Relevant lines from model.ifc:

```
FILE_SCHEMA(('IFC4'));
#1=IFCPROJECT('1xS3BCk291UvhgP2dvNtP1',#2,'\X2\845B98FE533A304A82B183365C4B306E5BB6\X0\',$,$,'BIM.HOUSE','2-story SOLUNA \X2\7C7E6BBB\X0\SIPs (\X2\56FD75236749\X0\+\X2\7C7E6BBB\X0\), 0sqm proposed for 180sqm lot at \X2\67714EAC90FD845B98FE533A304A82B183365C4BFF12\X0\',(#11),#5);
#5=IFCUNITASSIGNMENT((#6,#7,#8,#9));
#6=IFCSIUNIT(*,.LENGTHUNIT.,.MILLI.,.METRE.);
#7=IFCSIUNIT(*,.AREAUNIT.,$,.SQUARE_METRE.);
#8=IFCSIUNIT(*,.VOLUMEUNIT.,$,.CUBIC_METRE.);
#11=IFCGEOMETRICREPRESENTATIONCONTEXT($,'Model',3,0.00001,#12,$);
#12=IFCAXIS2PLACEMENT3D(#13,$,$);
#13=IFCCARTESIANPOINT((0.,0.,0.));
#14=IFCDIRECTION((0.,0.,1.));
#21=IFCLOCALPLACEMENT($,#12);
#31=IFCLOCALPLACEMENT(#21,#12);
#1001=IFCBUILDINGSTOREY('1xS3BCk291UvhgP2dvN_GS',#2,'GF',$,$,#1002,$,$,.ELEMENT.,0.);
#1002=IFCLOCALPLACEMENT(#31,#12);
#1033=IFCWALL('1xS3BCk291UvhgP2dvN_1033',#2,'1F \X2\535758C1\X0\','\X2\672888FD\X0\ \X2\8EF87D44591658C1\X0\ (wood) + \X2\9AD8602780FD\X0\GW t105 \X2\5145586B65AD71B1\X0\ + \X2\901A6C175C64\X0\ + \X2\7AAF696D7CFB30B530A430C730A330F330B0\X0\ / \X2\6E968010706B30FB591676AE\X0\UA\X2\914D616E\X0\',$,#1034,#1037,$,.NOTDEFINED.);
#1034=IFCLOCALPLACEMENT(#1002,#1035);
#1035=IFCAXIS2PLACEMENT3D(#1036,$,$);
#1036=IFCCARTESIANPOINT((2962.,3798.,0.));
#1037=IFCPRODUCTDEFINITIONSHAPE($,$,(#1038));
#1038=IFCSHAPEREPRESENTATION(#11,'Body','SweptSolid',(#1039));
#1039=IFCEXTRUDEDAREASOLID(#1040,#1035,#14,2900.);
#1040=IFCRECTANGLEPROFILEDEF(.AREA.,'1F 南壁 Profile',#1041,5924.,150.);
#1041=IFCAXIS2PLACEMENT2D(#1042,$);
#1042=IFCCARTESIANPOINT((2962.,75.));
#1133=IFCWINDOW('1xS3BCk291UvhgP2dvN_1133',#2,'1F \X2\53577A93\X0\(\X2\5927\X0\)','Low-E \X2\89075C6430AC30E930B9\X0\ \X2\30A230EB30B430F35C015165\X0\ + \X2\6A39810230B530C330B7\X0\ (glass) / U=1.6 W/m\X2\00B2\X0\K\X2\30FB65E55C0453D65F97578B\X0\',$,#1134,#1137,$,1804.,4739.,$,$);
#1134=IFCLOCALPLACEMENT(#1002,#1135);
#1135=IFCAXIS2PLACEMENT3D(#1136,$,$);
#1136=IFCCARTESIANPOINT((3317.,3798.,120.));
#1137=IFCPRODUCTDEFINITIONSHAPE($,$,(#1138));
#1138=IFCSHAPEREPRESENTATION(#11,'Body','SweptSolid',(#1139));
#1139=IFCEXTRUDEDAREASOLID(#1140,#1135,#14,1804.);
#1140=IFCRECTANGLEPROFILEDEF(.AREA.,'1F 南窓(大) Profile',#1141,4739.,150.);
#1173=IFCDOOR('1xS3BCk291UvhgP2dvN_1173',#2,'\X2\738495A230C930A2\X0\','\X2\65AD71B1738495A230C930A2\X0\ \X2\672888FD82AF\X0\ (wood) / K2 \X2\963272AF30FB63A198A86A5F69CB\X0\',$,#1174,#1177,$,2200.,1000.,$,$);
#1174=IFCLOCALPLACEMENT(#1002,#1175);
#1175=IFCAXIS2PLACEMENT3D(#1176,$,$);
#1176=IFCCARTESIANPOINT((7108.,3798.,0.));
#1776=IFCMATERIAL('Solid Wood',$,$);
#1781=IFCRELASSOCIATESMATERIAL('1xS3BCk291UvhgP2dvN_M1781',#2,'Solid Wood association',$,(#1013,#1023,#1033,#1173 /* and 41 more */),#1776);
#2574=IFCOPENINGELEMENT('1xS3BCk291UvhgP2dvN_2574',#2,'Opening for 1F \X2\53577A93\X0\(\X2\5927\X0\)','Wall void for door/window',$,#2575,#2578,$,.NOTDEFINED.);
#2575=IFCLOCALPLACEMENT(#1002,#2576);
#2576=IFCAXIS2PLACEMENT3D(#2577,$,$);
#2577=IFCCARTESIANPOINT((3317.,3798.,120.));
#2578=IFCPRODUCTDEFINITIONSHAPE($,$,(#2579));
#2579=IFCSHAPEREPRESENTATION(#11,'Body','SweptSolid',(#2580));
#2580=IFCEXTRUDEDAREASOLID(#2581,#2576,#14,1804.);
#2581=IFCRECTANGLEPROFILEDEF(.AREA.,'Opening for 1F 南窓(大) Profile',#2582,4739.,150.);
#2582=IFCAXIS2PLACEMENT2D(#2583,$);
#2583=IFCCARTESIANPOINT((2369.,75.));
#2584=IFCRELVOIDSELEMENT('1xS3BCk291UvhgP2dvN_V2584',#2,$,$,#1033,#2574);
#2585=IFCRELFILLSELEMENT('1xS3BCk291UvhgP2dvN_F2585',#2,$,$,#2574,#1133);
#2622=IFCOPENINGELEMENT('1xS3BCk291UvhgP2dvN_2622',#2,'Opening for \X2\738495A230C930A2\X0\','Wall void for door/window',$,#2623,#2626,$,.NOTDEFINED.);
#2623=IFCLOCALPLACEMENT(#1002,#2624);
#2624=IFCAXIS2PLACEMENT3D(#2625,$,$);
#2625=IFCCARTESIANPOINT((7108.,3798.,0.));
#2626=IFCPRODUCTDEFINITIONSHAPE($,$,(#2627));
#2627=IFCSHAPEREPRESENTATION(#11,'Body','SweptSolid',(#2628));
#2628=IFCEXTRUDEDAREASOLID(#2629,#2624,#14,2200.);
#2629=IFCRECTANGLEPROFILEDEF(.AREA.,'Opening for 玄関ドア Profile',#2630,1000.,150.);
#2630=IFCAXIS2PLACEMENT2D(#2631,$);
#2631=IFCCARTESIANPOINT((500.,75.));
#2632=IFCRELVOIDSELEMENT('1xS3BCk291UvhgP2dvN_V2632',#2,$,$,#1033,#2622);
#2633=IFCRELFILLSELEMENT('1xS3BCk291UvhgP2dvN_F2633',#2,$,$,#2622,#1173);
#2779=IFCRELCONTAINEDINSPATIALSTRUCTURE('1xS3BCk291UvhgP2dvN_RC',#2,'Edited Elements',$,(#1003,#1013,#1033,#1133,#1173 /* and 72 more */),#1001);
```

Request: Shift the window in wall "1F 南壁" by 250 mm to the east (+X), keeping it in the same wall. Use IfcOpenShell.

```python
import ifcopenshell
import ifcopenshell.api.geometry
import ifcopenshell.util.placement
import ifcopenshell.util.unit

model = ifcopenshell.open("model.ifc")
unit_scale = ifcopenshell.util.unit.calculate_unit_scale(model)

window = model.by_guid("1xS3BCk291UvhgP2dvN_1133")
opening = window.FillsVoids[0].RelatingOpeningElement
wall = opening.VoidsElements[0].RelatingBuildingElement

wall_matrix = ifcopenshell.util.placement.get_local_placement(wall.ObjectPlacement)
shift = wall_matrix[:3, 0] * 0.25 / unit_scale
before = ifcopenshell.util.placement.get_local_placement(window.ObjectPlacement)[:3, 3].copy()

# The window is not placed relative to its opening, so move both.
for product in (opening, window):
    matrix = ifcopenshell.util.placement.get_local_placement(product.ObjectPlacement)
    matrix[:3, 3] += shift
    ifcopenshell.api.geometry.edit_object_placement(model, product=product, matrix=matrix, is_si=False)

after = ifcopenshell.util.placement.get_local_placement(window.ObjectPlacement)[:3, 3]
print("window moved by", (after - before).round(3) + 0.0)

model.write("model_rev.ifc")
```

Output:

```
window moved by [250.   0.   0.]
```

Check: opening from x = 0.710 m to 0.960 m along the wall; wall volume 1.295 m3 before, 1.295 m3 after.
